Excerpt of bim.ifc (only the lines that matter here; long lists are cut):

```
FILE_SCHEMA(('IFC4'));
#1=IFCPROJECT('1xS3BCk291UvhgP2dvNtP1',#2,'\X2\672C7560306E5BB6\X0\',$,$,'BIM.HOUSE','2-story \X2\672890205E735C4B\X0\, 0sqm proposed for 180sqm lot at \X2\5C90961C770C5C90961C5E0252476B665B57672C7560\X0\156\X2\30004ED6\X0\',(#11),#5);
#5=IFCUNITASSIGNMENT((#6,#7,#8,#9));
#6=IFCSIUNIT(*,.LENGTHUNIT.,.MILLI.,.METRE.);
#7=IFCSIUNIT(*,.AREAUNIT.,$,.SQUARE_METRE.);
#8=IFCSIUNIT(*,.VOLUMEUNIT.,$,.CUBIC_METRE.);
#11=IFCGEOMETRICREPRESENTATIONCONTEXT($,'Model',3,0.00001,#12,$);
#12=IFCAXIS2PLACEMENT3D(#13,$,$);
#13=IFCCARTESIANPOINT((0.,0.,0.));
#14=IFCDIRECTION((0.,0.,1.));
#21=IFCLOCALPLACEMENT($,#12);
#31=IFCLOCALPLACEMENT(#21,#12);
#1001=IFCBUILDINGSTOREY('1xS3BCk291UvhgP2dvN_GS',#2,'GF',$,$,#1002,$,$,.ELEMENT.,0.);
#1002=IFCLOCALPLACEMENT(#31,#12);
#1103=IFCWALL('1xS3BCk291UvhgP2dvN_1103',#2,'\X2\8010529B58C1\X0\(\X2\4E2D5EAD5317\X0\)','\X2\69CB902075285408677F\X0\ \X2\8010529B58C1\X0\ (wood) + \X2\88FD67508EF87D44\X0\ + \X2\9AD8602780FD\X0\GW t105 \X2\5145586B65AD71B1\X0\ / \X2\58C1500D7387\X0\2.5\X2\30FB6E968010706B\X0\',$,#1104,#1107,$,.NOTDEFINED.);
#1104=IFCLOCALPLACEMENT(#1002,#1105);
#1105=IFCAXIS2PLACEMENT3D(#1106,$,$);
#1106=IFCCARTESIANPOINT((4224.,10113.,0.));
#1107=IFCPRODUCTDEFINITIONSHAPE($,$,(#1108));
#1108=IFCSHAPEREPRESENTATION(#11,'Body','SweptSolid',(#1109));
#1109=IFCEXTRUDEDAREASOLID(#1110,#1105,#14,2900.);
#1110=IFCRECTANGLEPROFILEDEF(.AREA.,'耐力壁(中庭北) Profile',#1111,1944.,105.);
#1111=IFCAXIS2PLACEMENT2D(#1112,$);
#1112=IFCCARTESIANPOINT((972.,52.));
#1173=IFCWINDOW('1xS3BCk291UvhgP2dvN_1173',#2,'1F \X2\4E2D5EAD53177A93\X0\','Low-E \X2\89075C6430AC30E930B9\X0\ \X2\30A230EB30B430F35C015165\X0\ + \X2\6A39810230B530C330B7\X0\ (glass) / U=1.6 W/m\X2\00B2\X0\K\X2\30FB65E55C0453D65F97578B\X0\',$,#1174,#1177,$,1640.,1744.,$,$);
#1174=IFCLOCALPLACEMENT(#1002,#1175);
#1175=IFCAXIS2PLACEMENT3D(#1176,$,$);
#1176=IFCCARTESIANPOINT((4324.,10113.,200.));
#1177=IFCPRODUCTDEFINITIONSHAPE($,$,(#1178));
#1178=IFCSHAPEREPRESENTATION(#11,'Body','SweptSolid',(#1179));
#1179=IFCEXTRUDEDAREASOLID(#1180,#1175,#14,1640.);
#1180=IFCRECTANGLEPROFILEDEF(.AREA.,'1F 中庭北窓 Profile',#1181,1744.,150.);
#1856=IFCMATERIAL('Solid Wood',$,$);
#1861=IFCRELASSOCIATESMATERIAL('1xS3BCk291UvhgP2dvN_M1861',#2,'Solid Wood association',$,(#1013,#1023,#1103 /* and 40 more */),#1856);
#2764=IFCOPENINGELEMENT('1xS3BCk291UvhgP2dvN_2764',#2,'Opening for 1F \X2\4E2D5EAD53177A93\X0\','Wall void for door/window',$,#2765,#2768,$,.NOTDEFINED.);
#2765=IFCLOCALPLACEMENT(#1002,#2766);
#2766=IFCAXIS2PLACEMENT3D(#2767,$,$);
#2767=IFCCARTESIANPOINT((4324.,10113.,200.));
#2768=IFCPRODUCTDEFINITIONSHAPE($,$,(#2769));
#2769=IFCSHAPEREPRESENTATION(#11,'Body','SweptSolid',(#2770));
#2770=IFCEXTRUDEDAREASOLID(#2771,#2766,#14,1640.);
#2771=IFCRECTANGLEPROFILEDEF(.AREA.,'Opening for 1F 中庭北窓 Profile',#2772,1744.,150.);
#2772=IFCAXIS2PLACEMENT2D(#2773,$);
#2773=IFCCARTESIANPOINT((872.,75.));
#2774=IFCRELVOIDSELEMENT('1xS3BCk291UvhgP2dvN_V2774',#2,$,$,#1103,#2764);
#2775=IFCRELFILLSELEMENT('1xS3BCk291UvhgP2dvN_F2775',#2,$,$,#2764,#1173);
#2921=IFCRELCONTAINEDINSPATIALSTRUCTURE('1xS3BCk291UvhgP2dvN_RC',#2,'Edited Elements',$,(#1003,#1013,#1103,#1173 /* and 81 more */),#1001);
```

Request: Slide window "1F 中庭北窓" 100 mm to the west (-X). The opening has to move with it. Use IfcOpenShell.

```python
import ifcopenshell
import ifcopenshell.api.geometry
import ifcopenshell.util.placement
import ifcopenshell.util.unit

model = ifcopenshell.open("bim.ifc")
unit_scale = ifcopenshell.util.unit.calculate_unit_scale(model)

window = model.by_guid("1xS3BCk291UvhgP2dvN_1173")
opening = window.FillsVoids[0].RelatingOpeningElement
wall = opening.VoidsElements[0].RelatingBuildingElement

wall_matrix = ifcopenshell.util.placement.get_local_placement(wall.ObjectPlacement)
shift = wall_matrix[:3, 0] * -0.1 / unit_scale
before = ifcopenshell.util.placement.get_local_placement(window.ObjectPlacement)[:3, 3].copy()

# The window is not placed relative to its opening, so move both.
for product in (opening, window):
    matrix = ifcopenshell.util.placement.get_local_placement(product.ObjectPlacement)
    matrix[:3, 3] += shift
    ifcopenshell.api.geometry.edit_object_placement(model, product=product, matrix=matrix, is_si=False)

after = ifcopenshell.util.placement.get_local_placement(window.ObjectPlacement)[:3, 3]
print("window moved by", (after - before).round(3) + 0.0)

model.write("bim_updated.ifc")
```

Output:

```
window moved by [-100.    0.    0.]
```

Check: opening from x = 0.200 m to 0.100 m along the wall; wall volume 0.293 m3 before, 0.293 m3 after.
